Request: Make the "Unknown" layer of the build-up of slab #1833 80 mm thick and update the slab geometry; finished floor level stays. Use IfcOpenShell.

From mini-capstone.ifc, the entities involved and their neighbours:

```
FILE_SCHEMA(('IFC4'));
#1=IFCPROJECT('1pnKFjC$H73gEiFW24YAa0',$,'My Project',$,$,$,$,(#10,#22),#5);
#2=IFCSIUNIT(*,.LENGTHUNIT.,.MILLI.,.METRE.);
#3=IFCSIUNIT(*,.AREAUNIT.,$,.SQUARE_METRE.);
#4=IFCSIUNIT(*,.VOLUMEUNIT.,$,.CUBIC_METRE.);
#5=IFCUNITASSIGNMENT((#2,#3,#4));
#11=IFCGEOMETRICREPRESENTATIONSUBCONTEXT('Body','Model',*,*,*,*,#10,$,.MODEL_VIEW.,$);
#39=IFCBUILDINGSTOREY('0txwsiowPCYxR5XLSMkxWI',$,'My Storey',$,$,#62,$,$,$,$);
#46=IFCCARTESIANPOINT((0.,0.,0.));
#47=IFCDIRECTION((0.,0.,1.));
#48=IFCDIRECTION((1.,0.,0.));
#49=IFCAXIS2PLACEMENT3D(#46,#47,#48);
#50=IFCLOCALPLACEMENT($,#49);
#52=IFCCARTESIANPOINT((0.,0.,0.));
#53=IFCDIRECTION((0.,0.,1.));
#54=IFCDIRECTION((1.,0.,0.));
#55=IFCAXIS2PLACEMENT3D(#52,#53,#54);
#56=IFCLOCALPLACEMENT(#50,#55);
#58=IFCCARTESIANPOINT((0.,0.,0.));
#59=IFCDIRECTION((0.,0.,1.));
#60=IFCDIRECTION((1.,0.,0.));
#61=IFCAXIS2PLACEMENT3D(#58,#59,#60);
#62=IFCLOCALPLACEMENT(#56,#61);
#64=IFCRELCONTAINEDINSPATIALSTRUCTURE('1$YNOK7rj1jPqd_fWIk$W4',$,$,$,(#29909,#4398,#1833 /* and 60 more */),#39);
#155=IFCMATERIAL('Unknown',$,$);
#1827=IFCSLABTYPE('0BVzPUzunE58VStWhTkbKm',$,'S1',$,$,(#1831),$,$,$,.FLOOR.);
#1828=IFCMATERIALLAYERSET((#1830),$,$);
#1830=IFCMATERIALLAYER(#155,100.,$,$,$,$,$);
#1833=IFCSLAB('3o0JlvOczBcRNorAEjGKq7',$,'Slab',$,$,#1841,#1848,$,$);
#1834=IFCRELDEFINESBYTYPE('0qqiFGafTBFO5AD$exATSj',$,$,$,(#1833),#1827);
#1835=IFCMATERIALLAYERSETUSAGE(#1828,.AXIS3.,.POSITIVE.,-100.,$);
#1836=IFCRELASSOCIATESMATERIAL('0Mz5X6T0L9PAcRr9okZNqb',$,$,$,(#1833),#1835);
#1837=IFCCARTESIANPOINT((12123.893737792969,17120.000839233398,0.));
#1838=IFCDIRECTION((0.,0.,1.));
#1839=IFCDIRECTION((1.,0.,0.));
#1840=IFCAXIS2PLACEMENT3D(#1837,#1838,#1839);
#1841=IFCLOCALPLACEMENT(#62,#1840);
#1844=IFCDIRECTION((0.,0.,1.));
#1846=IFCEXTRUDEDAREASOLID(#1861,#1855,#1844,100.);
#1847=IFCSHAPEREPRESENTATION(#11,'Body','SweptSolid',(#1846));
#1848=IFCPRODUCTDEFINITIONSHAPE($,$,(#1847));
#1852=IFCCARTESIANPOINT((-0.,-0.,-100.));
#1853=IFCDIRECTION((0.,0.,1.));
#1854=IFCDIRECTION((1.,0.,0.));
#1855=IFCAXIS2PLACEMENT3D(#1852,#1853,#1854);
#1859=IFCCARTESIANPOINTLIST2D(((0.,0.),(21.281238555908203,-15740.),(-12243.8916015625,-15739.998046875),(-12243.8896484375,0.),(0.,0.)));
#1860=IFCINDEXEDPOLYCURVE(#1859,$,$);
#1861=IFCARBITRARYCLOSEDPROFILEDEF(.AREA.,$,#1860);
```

```python
import ifcopenshell
import ifcopenshell.util.element
import ifcopenshell.util.representation
import ifcopenshell.util.unit

model = ifcopenshell.open("mini-capstone.ifc")
unit_scale = ifcopenshell.util.unit.calculate_unit_scale(model)

layer_set = model.by_id(1828)
layer = next(l for l in layer_set.MaterialLayers if l.Material and l.Material.Name == "Unknown")
change = 0.08 / unit_scale - layer.LayerThickness
layer.LayerThickness += change

# Geometry does not follow the layer set by itself.
slabs = [e for e in ifcopenshell.util.element.get_elements_by_material(model, layer_set) if e.is_a("IfcSlab")]
for slab in sorted(slabs, key=lambda e: e.id()):
    body = ifcopenshell.util.representation.get_representation(slab, "Model", "Body")
    solid = body.Items[0]
    old_depth = solid.Depth
    solid.Depth += change
    # Extruded upwards: lower the start of the extrusion so the top stays.
    x, y, z = solid.Position.Location.Coordinates
    solid.Position.Location = model.createIfcCartesianPoint((x, y, z - change))
    print(slab.id(), f"{old_depth:g} -> {solid.Depth:g}")

# The layers are counted up from the underside, which has moved.
for usage in {ifcopenshell.util.element.get_material(slab) for slab in slabs}:
    usage.OffsetFromReferenceLine -= change

model.write("mini-capstone_rev.ifc")
```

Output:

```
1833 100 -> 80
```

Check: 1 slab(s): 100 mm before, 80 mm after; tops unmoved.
